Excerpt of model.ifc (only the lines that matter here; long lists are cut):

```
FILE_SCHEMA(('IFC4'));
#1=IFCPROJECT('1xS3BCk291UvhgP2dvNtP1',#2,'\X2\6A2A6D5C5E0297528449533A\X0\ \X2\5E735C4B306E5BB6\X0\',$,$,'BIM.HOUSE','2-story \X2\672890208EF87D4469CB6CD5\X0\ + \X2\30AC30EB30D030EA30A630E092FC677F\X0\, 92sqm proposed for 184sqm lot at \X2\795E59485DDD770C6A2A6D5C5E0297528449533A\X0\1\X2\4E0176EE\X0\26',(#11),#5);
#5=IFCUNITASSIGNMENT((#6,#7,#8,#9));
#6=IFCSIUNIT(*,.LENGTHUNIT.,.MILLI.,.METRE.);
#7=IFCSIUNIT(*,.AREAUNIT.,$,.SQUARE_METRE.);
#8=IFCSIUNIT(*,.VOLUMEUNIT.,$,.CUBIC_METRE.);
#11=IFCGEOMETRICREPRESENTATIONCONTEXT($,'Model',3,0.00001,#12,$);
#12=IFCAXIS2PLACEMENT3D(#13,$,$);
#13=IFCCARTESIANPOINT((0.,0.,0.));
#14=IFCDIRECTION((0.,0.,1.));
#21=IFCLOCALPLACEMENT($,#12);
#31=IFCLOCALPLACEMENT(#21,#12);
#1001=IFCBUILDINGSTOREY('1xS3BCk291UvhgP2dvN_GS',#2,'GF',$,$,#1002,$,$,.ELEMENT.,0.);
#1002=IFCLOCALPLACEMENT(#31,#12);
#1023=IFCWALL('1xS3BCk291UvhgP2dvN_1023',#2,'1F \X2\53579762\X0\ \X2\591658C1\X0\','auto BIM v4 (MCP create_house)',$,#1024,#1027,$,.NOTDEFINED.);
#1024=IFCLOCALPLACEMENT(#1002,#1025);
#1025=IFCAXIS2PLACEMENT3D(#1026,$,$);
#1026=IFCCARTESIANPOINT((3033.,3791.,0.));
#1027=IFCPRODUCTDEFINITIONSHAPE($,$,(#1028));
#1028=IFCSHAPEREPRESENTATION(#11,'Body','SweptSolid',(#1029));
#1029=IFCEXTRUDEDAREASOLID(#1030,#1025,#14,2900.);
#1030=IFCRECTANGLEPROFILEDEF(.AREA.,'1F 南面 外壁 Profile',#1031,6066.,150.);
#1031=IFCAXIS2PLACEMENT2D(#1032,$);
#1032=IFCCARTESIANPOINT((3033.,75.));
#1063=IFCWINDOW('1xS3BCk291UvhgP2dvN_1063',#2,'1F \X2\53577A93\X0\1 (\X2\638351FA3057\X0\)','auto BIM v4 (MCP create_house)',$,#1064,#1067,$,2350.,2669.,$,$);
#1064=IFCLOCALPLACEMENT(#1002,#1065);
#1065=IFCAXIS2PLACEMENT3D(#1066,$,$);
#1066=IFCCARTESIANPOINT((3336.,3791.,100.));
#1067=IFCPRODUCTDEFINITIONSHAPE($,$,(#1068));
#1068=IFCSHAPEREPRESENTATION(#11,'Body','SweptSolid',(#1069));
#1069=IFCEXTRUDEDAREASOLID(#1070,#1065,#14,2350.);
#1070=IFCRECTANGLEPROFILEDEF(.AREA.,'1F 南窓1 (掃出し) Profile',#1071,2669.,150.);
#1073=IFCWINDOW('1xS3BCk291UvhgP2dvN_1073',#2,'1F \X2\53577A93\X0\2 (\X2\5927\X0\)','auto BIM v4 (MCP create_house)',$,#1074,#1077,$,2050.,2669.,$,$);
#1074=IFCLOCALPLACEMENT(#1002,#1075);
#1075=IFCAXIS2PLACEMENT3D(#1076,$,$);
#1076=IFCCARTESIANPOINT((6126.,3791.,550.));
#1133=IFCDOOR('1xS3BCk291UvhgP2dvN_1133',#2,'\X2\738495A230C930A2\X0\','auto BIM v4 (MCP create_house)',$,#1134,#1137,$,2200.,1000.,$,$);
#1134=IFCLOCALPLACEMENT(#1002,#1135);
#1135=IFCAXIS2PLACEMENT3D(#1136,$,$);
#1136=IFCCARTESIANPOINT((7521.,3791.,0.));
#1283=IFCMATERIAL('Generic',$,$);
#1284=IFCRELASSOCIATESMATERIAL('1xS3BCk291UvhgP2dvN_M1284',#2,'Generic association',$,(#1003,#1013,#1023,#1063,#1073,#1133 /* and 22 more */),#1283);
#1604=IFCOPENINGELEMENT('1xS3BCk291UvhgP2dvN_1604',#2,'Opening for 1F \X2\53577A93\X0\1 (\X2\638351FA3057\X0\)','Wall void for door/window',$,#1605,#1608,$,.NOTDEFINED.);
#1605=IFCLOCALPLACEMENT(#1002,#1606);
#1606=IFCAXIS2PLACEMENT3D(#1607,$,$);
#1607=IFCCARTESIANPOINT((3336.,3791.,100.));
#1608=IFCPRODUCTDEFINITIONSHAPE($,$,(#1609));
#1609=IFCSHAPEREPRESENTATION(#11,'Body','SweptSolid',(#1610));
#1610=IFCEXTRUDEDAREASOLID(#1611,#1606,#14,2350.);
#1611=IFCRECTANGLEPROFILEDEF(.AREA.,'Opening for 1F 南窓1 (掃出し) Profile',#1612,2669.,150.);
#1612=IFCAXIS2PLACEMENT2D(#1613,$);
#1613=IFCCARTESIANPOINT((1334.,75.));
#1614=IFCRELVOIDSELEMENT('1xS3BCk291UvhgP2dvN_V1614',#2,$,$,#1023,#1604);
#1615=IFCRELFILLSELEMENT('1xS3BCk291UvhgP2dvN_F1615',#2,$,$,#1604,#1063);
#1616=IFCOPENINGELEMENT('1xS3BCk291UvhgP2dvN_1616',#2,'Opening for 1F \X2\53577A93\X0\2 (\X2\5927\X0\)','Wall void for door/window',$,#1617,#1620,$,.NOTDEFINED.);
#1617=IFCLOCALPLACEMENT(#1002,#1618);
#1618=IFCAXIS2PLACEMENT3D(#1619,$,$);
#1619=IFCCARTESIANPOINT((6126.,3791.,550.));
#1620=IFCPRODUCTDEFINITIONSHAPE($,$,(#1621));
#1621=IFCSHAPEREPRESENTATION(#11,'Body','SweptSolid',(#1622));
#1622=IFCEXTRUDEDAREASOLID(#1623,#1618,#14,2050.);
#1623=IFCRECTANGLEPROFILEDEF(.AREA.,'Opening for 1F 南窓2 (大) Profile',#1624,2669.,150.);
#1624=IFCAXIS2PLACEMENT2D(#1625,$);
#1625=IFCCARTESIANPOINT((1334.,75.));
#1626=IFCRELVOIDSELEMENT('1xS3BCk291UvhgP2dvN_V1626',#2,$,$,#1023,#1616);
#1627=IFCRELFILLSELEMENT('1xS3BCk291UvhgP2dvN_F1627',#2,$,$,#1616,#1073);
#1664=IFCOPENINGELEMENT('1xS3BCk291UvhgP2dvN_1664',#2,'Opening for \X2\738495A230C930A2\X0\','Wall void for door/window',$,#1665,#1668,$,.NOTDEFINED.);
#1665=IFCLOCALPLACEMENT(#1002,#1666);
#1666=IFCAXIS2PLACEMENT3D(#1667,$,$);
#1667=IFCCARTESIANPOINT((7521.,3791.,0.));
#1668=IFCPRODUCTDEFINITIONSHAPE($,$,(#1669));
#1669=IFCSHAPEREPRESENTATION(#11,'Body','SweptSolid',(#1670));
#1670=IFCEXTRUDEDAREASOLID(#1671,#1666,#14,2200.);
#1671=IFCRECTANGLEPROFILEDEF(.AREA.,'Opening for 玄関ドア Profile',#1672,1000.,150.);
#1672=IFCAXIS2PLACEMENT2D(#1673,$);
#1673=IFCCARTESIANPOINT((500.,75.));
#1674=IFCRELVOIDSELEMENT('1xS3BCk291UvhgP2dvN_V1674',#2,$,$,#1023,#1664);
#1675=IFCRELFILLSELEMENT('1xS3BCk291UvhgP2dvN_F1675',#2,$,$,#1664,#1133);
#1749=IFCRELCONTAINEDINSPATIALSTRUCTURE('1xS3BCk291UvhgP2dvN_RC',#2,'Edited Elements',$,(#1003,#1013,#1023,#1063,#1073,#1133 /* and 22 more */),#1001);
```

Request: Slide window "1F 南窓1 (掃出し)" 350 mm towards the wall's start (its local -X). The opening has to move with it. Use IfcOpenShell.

```python
import ifcopenshell
import ifcopenshell.api.geometry
import ifcopenshell.util.placement

model = ifcopenshell.open("model.ifc")

window = model.by_id(1063)
opening = window.FillsVoids[0].RelatingOpeningElement
wall = opening.VoidsElements[0].RelatingBuildingElement

wall_matrix = ifcopenshell.util.placement.get_local_placement(wall.ObjectPlacement)
shift = wall_matrix[:3, 0] * -350.0
before = ifcopenshell.util.placement.get_local_placement(window.ObjectPlacement)[:3, 3].copy()

# The window is not placed relative to its opening, so move both.
for product in (opening, window):
    matrix = ifcopenshell.util.placement.get_local_placement(product.ObjectPlacement)
    matrix[:3, 3] += shift
    ifcopenshell.api.geometry.edit_object_placement(model, product=product, matrix=matrix, is_si=False)

after = ifcopenshell.util.placement.get_local_placement(window.ObjectPlacement)[:3, 3]
print("window moved by", (after - before).round(3) + 0.0)

model.write("model_updated.ifc")
```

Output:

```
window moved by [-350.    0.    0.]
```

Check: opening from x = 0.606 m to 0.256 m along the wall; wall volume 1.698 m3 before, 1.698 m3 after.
